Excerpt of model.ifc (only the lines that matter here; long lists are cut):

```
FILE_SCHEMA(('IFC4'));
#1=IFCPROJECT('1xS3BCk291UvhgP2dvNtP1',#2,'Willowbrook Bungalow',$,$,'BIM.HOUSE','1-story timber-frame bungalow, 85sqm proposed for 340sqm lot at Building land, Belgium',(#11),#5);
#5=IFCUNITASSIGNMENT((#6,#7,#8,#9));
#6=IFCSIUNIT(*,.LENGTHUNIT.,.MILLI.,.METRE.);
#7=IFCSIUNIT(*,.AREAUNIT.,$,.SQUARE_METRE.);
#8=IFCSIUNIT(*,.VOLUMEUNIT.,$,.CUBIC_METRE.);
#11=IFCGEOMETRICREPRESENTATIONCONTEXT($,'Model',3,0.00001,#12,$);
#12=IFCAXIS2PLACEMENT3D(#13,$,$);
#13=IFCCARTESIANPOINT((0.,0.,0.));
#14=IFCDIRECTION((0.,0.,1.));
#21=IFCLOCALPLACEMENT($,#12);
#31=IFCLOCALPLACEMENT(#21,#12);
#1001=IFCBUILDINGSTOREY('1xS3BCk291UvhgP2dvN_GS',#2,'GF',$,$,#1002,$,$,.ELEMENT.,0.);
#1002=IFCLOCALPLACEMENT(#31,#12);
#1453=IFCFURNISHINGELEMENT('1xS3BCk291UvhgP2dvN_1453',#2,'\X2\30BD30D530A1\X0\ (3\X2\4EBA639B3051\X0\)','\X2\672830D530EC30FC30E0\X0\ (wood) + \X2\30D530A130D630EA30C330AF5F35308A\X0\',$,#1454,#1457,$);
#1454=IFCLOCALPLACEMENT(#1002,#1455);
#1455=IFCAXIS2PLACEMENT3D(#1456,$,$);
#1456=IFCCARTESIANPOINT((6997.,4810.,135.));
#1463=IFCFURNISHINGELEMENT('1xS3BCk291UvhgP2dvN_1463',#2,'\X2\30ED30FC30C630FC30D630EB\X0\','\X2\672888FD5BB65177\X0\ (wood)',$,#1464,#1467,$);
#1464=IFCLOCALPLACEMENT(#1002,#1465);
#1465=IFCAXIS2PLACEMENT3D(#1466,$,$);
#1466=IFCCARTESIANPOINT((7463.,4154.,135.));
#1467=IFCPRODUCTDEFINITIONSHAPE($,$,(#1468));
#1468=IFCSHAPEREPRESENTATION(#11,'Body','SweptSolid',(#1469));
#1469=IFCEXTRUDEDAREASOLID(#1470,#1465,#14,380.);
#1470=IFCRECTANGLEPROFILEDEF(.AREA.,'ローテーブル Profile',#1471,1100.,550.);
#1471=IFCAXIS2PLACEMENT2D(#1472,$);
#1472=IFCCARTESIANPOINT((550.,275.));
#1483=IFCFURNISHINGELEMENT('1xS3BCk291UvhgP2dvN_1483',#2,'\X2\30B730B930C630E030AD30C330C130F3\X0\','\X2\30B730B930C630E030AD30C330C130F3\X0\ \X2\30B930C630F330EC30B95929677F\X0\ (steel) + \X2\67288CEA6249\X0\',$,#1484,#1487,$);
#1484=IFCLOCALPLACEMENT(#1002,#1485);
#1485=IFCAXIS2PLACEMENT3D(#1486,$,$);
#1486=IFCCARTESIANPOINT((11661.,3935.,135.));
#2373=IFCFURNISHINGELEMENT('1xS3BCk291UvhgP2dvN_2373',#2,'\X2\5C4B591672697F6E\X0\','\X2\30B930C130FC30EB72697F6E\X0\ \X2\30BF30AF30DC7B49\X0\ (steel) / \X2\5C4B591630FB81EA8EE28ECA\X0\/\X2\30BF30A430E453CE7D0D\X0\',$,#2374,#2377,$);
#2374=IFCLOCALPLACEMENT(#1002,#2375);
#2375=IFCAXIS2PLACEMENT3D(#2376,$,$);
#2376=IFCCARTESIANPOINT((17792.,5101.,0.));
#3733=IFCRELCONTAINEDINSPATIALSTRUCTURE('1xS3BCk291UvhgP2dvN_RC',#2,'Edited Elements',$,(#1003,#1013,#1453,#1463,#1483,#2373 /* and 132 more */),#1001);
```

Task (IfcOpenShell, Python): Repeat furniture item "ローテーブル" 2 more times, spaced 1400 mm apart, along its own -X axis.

```python
import ifcopenshell
import ifcopenshell.api.geometry
import ifcopenshell.api.root
import ifcopenshell.util.element
import ifcopenshell.util.placement

model = ifcopenshell.open("model.ifc")


def reuse_history(source, copy):
    """copy_class also copies each property set's owner history, people and application; keep the originals."""
    for rel in copy.IsDefinedBy:
        if rel.is_a("IfcRelDefinesByProperties") and (history := rel.RelatingPropertyDefinition.OwnerHistory):
            rel.RelatingPropertyDefinition.OwnerHistory = source.OwnerHistory
            ifcopenshell.util.element.remove_deep2(model, history)


source = model.by_id(1463)
base = ifcopenshell.util.placement.get_local_placement(source.ObjectPlacement)
step = -base[:3, 0] * 1400.0

for i in range(1, 3):
    copy = ifcopenshell.api.root.copy_class(model, product=source)
    copy.Representation = ifcopenshell.util.element.copy_deep(
        model, source.Representation, exclude=["IfcGeometricRepresentationContext", "IfcRepresentationMap"]
    )
    reuse_history(source, copy)
    matrix = base.copy()
    matrix[:3, 3] += i * step
    print("added at", matrix[:3, 3].round(3) + 0.0)
    ifcopenshell.api.geometry.edit_object_placement(model, product=copy, matrix=matrix, is_si=False)

model.write("model_rev.ifc")
```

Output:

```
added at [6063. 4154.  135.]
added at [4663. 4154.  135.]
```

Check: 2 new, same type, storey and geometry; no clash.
